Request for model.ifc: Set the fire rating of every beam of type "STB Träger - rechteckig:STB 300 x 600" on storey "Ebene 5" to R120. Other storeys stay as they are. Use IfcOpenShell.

First a look at what the model holds.

```python
import ifcopenshell
import ifcopenshell.util.element

model = ifcopenshell.open("model.ifc")
print(model.schema)
storey = next(s for s in model.by_type("IfcBuildingStorey") if s.Name == "Ebene 5")
beams = [e for e in ifcopenshell.util.element.get_decomposition(storey) if e.is_a("IfcBeam")]
seen = {}
for e in beams:
    element_type = ifcopenshell.util.element.get_type(e)
    key = (element_type.Name if element_type != e and element_type else None, ifcopenshell.util.element.get_pset(e, "Pset_BeamCommon", "FireRating"))
    seen[key] = seen.get(key, 0) + 1
for (name, value), count in sorted(seen.items(), key=str):
    print(count, "x", name, "|", value)
```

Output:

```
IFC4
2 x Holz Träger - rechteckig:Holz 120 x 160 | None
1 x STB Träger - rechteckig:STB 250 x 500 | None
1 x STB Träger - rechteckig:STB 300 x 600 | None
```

```python
import ifcopenshell
import ifcopenshell.api.pset
import ifcopenshell.util.element

model = ifcopenshell.open("model.ifc")

storey = next(s for s in model.by_type("IfcBuildingStorey") if s.Name == "Ebene 5")
beams = [e for e in ifcopenshell.util.element.get_decomposition(storey) if e.is_a("IfcBeam")]

count = 0
for e in beams:
    element_type = ifcopenshell.util.element.get_type(e)
    if element_type in (None, e) or element_type.Name != "STB Träger - rechteckig:STB 300 x 600":
        continue
    # add_pset returns the element's existing set when there is one.
    pset = ifcopenshell.api.pset.add_pset(model, product=e, name="Pset_BeamCommon")
    ifcopenshell.api.pset.edit_pset(model, pset=pset, properties={"FireRating": "R120"})
    count += 1

print(count, "beams updated")

model.write("model_edited.ifc")
```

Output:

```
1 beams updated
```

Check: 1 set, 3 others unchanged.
